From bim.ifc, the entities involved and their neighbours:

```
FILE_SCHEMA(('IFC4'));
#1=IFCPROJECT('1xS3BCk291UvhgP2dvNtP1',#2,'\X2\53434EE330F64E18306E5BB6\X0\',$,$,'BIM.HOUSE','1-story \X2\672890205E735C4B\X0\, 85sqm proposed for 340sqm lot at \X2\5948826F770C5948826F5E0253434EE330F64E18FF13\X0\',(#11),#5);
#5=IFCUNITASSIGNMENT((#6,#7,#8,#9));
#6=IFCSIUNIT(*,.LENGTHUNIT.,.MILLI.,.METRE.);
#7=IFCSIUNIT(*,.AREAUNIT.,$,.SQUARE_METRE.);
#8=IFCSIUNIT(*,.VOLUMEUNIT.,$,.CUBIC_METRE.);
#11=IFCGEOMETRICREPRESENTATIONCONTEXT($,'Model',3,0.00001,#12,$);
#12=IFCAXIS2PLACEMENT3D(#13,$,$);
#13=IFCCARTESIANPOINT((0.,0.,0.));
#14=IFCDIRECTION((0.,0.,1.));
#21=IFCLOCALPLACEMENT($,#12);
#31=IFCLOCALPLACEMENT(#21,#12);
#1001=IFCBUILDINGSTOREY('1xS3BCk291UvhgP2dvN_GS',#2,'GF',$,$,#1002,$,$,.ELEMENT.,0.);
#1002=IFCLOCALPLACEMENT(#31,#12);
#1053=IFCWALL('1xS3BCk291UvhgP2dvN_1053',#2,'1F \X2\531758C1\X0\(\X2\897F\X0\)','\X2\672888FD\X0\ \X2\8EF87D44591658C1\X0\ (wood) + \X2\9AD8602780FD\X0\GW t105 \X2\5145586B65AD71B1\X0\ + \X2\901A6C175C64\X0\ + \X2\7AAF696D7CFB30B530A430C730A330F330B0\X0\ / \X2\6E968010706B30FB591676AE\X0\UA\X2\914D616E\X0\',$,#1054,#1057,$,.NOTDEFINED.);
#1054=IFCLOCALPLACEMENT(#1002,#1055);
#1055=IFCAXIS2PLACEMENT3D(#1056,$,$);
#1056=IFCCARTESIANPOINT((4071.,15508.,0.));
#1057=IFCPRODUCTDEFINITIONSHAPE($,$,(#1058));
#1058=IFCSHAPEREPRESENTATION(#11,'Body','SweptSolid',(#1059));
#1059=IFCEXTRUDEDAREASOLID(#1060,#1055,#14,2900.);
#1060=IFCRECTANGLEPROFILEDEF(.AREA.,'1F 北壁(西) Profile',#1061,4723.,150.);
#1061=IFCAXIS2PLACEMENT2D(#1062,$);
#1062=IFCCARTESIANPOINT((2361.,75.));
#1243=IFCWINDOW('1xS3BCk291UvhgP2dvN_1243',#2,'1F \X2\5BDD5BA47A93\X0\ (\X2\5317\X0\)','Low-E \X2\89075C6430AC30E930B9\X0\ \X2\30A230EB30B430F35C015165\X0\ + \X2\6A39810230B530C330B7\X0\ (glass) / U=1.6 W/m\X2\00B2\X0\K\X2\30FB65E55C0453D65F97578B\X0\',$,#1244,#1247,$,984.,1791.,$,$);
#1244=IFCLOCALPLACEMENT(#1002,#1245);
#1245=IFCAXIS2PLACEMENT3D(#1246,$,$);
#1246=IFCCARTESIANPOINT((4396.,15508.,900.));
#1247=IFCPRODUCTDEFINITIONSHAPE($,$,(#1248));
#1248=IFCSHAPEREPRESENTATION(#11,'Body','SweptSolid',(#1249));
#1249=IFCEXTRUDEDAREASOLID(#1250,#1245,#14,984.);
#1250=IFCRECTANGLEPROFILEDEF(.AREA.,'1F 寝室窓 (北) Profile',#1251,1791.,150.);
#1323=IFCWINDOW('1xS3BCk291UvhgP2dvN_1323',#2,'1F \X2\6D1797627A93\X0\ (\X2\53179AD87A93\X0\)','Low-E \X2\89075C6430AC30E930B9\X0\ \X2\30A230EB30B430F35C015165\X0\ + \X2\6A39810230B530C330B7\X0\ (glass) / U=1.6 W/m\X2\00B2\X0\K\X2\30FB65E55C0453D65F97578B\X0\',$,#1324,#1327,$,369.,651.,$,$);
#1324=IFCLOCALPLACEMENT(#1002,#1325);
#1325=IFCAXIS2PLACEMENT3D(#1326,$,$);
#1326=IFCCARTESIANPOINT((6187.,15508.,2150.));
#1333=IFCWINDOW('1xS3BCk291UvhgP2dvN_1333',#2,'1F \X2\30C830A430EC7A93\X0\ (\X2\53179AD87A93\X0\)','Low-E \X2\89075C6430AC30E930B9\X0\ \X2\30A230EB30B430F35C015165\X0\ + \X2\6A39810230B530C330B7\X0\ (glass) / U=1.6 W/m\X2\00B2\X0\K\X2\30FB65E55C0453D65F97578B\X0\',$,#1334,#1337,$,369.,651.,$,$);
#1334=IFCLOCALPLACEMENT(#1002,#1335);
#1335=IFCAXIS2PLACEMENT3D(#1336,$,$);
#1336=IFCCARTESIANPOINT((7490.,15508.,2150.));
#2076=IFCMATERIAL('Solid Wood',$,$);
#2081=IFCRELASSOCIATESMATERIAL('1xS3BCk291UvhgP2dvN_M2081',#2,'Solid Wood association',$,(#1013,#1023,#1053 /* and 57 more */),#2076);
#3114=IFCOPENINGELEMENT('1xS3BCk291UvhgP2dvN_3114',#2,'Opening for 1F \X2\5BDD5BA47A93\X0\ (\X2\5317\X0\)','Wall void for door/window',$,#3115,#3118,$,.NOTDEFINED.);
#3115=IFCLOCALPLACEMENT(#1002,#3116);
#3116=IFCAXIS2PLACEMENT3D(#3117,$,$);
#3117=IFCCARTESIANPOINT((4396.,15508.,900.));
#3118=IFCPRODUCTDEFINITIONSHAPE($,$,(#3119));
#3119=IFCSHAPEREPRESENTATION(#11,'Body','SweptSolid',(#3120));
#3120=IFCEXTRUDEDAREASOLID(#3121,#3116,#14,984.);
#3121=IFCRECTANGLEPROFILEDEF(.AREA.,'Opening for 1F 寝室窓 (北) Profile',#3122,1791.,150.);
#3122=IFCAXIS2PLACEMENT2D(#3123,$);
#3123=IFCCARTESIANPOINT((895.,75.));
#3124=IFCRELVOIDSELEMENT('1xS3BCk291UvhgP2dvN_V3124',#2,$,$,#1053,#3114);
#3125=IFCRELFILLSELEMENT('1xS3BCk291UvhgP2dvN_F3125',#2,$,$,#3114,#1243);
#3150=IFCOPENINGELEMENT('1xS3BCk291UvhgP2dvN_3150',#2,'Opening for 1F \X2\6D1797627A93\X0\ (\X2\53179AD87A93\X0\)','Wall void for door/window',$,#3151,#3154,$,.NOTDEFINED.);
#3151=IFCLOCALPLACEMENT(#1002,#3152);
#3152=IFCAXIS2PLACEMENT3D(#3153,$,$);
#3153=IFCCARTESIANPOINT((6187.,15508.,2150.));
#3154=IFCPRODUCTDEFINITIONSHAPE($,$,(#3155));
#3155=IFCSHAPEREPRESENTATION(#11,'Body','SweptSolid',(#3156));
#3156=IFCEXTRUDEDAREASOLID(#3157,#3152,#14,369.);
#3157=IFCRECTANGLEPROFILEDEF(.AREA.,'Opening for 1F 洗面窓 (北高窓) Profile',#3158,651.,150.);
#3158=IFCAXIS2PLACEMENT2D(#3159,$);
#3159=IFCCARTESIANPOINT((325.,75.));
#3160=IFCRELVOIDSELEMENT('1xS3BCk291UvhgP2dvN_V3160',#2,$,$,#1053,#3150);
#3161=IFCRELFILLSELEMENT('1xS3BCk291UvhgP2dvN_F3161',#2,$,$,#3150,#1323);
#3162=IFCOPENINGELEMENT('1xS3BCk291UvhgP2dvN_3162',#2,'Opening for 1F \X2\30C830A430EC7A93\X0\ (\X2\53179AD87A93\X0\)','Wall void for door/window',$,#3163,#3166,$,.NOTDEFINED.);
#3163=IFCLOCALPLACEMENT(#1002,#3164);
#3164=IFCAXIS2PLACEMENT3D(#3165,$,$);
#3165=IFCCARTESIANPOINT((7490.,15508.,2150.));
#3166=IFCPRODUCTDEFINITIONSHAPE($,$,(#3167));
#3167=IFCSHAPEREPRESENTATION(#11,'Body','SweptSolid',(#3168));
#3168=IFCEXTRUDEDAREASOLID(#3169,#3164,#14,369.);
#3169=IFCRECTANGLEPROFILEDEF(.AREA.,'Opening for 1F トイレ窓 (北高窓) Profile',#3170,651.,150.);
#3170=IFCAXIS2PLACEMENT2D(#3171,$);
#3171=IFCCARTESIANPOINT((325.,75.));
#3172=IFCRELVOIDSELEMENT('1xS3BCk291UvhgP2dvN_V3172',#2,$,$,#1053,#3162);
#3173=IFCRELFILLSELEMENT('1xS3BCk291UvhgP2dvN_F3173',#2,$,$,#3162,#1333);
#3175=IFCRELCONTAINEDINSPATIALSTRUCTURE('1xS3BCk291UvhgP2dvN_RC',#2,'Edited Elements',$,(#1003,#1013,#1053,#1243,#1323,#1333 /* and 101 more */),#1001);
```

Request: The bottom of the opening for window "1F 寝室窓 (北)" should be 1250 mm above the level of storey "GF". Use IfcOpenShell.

```python
import numpy as np
import ifcopenshell
import ifcopenshell.api.geometry
import ifcopenshell.geom
import ifcopenshell.util.element
import ifcopenshell.util.placement
import ifcopenshell.util.shape
import ifcopenshell.util.unit

model = ifcopenshell.open("bim.ifc")
unit_scale = ifcopenshell.util.unit.calculate_unit_scale(model)

window = model.by_guid("1xS3BCk291UvhgP2dvN_1243")
opening = window.FillsVoids[0].RelatingOpeningElement
storey = ifcopenshell.util.element.get_container(window, ifc_class="IfcBuildingStorey")
level = ifcopenshell.util.placement.get_local_placement(storey.ObjectPlacement)[2, 3]

# The opening's origin need not be at the sill, so measure its lowest point.
shape = ifcopenshell.geom.create_shape(ifcopenshell.geom.settings(), opening)
bottom = ifcopenshell.util.shape.get_shape_bottom_elevation(shape, shape.geometry) / unit_scale
dz = level + 1.25 / unit_scale - bottom

shift = np.array([0.0, 0.0, dz])
# The window is not placed relative to its opening, so move both.
for product in (opening, window):
    matrix = ifcopenshell.util.placement.get_local_placement(product.ObjectPlacement)
    matrix[:3, 3] += shift
    ifcopenshell.api.geometry.edit_object_placement(model, product=product, matrix=matrix, is_si=False)

print(f"moved by {dz * unit_scale:+.3f} m")

model.write("bim_updated.ifc")
```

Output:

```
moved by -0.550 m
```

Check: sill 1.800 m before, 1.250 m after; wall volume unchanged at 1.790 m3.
